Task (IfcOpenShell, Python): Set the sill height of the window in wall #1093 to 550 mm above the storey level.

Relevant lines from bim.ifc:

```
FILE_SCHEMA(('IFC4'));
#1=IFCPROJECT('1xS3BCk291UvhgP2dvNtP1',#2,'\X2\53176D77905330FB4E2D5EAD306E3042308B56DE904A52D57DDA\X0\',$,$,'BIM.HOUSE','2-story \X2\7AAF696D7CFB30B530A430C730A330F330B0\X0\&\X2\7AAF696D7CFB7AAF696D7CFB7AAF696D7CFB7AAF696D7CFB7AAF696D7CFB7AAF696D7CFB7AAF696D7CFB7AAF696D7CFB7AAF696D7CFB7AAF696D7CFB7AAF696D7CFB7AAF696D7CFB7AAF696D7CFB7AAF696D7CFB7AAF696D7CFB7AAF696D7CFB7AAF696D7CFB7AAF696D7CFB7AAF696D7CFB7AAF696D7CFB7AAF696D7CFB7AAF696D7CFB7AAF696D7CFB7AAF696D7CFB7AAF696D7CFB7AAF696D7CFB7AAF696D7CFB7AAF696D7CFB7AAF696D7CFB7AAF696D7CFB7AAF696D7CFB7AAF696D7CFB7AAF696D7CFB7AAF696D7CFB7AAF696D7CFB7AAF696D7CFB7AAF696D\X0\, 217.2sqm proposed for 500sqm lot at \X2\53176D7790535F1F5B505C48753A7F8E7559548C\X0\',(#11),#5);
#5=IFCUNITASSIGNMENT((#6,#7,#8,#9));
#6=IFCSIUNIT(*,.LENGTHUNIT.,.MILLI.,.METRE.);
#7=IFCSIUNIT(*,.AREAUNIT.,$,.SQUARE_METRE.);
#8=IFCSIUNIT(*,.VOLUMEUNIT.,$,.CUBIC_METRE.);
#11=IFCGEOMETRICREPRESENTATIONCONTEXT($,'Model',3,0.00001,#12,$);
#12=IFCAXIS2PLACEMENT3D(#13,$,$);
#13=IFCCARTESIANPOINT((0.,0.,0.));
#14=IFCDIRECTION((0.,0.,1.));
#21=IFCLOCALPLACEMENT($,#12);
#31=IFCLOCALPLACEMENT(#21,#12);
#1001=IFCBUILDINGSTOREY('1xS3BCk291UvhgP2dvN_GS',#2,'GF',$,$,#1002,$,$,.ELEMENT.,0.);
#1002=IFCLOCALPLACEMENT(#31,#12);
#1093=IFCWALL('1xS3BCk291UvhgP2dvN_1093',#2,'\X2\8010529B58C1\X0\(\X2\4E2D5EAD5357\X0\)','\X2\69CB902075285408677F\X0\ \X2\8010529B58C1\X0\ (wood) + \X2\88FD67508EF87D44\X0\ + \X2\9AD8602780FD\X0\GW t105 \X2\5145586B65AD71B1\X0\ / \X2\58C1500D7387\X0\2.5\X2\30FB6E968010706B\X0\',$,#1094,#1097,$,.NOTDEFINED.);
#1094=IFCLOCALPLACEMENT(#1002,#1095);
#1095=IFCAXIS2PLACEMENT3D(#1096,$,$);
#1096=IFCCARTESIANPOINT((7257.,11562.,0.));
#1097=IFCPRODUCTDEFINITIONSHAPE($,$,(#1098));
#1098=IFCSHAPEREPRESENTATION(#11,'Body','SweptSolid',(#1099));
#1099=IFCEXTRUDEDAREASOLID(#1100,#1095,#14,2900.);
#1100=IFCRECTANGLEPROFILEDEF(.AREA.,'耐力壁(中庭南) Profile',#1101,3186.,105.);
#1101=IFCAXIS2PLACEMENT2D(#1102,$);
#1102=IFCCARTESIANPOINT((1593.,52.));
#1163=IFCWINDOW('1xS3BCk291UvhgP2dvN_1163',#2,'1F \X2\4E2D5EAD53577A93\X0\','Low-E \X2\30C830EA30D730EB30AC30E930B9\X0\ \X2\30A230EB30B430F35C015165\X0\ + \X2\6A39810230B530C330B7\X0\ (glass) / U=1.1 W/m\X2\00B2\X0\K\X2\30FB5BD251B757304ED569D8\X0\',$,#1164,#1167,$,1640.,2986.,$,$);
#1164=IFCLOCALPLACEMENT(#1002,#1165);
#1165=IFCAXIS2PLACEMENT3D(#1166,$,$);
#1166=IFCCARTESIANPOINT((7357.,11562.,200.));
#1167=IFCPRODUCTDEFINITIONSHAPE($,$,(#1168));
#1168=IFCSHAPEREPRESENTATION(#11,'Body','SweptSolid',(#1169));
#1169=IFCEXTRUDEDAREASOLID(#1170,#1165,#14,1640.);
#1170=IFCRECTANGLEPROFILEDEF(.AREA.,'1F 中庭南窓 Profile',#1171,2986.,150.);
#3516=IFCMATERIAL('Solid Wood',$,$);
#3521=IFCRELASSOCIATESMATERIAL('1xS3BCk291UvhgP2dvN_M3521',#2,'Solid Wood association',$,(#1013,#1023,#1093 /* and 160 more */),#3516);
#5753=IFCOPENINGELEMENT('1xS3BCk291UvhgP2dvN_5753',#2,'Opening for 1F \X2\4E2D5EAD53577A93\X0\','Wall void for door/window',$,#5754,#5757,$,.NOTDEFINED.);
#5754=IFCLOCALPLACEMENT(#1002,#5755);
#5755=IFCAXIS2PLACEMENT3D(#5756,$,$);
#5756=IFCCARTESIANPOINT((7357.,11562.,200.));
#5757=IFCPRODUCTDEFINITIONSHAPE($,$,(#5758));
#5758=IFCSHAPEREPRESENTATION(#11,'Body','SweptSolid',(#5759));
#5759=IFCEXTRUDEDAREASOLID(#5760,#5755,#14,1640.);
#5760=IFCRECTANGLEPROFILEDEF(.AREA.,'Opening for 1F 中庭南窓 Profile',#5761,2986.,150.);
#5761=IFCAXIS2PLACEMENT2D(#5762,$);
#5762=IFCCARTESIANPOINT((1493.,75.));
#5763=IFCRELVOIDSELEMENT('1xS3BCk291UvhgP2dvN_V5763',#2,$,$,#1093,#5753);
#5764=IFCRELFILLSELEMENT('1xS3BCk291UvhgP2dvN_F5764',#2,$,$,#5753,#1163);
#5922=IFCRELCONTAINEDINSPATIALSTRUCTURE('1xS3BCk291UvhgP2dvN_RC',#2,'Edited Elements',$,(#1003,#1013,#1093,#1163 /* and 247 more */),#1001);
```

```python
import numpy as np
import ifcopenshell
import ifcopenshell.api.geometry
import ifcopenshell.geom
import ifcopenshell.util.element
import ifcopenshell.util.placement
import ifcopenshell.util.shape
import ifcopenshell.util.unit

model = ifcopenshell.open("bim.ifc")
unit_scale = ifcopenshell.util.unit.calculate_unit_scale(model)

window = model.by_id(1163)
opening = window.FillsVoids[0].RelatingOpeningElement
storey = ifcopenshell.util.element.get_container(window, ifc_class="IfcBuildingStorey")
level = ifcopenshell.util.placement.get_local_placement(storey.ObjectPlacement)[2, 3]

# The opening's origin need not be at the sill, so measure its lowest point.
shape = ifcopenshell.geom.create_shape(ifcopenshell.geom.settings(), opening)
bottom = ifcopenshell.util.shape.get_shape_bottom_elevation(shape, shape.geometry) / unit_scale
dz = level + 0.55 / unit_scale - bottom

shift = np.array([0.0, 0.0, dz])
# The window is not placed relative to its opening, so move both.
for product in (opening, window):
    matrix = ifcopenshell.util.placement.get_local_placement(product.ObjectPlacement)
    matrix[:3, 3] += shift
    ifcopenshell.api.geometry.edit_object_placement(model, product=product, matrix=matrix, is_si=False)

print(f"moved by {dz * unit_scale:+.3f} m")

model.write("bim-out.ifc")
```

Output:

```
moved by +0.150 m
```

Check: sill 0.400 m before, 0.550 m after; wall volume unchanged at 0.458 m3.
